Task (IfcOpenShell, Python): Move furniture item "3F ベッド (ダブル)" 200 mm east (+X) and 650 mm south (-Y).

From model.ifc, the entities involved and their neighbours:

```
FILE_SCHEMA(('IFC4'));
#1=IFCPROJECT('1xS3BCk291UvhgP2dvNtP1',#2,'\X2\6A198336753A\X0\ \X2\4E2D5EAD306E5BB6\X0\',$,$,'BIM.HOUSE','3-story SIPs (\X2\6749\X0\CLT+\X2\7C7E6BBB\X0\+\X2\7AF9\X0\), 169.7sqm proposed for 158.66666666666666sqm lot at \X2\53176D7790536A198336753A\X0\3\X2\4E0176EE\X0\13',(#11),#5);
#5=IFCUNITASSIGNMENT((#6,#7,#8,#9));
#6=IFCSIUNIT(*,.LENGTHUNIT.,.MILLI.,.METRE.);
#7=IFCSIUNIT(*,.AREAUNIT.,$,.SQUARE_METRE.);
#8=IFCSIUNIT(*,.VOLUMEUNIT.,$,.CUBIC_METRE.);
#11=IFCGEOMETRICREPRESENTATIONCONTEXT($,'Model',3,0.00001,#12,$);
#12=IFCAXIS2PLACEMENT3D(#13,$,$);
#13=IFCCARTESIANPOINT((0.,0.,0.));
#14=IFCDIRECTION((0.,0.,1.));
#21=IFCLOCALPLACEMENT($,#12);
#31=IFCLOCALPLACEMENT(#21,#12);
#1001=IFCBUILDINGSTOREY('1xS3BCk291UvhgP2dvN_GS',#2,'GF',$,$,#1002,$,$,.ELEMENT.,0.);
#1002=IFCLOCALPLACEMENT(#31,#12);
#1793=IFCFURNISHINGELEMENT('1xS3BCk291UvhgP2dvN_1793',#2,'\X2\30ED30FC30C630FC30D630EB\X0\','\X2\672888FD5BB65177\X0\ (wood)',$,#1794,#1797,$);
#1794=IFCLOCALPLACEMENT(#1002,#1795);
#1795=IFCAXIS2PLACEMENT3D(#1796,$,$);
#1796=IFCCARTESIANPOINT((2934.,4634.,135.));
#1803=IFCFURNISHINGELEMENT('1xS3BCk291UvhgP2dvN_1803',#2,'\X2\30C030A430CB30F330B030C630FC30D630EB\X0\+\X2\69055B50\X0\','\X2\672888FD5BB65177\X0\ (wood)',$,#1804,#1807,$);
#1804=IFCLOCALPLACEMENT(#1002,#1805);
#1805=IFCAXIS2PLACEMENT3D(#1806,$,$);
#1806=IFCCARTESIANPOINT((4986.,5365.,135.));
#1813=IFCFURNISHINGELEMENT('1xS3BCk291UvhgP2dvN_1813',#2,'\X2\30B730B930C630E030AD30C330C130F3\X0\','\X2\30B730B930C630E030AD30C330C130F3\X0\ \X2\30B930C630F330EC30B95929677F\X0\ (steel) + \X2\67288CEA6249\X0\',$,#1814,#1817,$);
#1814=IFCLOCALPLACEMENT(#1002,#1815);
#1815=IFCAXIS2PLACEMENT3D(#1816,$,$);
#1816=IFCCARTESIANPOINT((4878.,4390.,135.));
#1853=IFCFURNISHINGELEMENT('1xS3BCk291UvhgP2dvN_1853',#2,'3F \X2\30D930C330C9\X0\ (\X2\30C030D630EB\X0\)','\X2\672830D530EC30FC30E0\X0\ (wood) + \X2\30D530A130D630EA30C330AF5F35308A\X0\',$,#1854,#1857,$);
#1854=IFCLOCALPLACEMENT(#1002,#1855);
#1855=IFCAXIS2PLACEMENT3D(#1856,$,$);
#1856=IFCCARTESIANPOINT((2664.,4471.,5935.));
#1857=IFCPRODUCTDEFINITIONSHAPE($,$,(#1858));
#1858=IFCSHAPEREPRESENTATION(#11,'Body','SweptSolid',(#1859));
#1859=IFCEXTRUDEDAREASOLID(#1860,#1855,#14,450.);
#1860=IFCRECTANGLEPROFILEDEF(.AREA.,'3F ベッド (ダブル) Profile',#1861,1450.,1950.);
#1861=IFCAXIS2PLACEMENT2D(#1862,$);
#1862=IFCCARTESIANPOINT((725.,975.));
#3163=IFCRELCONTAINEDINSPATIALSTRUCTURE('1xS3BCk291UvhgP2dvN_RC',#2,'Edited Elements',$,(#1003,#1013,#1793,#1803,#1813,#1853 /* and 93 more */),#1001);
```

```python
import ifcopenshell
import ifcopenshell.api.geometry
import ifcopenshell.util.placement
import ifcopenshell.util.unit

model = ifcopenshell.open("model.ifc")
unit_scale = ifcopenshell.util.unit.calculate_unit_scale(model)

item = model.by_guid("1xS3BCk291UvhgP2dvN_1853")
matrix = ifcopenshell.util.placement.get_local_placement(item.ObjectPlacement)
matrix[0, 3] += 0.2 / unit_scale
matrix[1, 3] -= 0.65 / unit_scale
ifcopenshell.api.geometry.edit_object_placement(model, product=item, matrix=matrix, is_si=False)

print(ifcopenshell.util.placement.get_local_placement(item.ObjectPlacement).round(3) + 0.0)

model.write("model_edited.ifc")
```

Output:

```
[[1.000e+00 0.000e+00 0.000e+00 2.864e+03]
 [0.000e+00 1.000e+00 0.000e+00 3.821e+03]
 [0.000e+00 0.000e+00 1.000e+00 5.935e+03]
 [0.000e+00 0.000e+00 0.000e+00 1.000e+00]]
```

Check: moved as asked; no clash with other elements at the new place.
